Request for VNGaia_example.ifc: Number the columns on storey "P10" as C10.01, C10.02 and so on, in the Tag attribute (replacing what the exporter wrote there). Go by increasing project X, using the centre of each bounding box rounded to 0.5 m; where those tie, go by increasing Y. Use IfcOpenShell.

First a look at what the model holds.

```python
import ifcopenshell
import ifcopenshell.util.element
import ifcopenshell.util.placement

model = ifcopenshell.open("VNGaia_example.ifc")
print(model.schema)
storey = next(s for s in model.by_type("IfcBuildingStorey") if s.Name == "P10")
columns = [e for e in ifcopenshell.util.element.get_decomposition(storey) if e.is_a("IfcColumn")]
for e in sorted(columns, key=lambda e: e.id()):
    origin = ifcopenshell.util.placement.get_local_placement(e.ObjectPlacement)[:3, 3]
    print(e.id(), e.Tag, e.Name, origin.round(2) + 0.0, sep=" | ")
```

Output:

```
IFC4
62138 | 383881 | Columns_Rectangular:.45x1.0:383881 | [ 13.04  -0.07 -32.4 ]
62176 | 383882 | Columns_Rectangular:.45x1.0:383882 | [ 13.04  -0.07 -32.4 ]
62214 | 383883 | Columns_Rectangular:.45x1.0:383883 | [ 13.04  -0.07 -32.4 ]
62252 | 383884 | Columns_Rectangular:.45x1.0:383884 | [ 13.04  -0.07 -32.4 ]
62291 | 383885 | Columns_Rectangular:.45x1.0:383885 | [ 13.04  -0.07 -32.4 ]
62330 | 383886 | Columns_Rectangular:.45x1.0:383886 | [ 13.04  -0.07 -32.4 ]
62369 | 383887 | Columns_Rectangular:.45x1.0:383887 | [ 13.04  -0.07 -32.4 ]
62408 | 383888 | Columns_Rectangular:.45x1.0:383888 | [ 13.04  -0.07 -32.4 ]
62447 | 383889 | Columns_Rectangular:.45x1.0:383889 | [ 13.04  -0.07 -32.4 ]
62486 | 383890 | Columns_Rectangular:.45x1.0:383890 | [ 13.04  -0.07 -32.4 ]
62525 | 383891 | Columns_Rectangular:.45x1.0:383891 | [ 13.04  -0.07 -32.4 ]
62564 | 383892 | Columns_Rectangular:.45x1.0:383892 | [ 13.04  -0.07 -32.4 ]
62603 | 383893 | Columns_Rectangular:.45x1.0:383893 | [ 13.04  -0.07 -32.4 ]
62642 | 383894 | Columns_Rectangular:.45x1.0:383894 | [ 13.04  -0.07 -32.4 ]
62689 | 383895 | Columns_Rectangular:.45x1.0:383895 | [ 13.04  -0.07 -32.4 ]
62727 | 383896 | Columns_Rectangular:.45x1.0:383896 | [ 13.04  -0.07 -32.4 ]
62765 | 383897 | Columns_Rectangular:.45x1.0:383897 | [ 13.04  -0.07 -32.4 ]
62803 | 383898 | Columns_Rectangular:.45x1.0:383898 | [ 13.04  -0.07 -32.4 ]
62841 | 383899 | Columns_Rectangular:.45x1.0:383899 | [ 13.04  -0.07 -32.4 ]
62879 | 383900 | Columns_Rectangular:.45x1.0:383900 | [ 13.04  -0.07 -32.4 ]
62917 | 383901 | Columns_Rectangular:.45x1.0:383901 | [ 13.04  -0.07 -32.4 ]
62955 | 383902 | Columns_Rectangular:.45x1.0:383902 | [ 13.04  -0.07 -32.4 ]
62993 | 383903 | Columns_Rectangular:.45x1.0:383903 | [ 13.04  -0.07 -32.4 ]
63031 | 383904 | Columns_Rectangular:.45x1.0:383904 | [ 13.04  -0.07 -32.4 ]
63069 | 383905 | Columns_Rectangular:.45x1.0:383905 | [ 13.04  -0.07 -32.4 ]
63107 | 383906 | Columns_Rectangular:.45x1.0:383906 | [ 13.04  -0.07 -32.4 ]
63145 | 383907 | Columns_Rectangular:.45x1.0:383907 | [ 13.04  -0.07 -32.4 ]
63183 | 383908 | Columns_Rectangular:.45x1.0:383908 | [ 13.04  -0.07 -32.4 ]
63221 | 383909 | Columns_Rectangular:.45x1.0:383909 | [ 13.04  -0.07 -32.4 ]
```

```python
import ifcopenshell
import ifcopenshell.geom
import ifcopenshell.util.element
import ifcopenshell.util.shape

model = ifcopenshell.open("VNGaia_example.ifc")
settings = ifcopenshell.geom.settings()
settings.set("use-world-coords", True)


def centre(element):
    shape = ifcopenshell.geom.create_shape(settings, element)
    return ifcopenshell.util.shape.get_bbox_centroid(shape.geometry)


storey = next(s for s in model.by_type("IfcBuildingStorey") if s.Name == "P10")
columns = [e for e in ifcopenshell.util.element.get_decomposition(storey) if e.is_a("IfcColumn")]

# Insertion points can sit at a corner or the storey origin, so sort by the geometry (in metres).
centres = {e: centre(e) for e in columns}
columns.sort(key=lambda e: (round(centres[e][0] / 0.5), centres[e][1]))

for i, e in enumerate(columns, start=1):
    number = f"C10.{i:02d}"
    e.Tag = number
    print(e.id(), number)

model.write("VNGaia_example_v2.ifc")
```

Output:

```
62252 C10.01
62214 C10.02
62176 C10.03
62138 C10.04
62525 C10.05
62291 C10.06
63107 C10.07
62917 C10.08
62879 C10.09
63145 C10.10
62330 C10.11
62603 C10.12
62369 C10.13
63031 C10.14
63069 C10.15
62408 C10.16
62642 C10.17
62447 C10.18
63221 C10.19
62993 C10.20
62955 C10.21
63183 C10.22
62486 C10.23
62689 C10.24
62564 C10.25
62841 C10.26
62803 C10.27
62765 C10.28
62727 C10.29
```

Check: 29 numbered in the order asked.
